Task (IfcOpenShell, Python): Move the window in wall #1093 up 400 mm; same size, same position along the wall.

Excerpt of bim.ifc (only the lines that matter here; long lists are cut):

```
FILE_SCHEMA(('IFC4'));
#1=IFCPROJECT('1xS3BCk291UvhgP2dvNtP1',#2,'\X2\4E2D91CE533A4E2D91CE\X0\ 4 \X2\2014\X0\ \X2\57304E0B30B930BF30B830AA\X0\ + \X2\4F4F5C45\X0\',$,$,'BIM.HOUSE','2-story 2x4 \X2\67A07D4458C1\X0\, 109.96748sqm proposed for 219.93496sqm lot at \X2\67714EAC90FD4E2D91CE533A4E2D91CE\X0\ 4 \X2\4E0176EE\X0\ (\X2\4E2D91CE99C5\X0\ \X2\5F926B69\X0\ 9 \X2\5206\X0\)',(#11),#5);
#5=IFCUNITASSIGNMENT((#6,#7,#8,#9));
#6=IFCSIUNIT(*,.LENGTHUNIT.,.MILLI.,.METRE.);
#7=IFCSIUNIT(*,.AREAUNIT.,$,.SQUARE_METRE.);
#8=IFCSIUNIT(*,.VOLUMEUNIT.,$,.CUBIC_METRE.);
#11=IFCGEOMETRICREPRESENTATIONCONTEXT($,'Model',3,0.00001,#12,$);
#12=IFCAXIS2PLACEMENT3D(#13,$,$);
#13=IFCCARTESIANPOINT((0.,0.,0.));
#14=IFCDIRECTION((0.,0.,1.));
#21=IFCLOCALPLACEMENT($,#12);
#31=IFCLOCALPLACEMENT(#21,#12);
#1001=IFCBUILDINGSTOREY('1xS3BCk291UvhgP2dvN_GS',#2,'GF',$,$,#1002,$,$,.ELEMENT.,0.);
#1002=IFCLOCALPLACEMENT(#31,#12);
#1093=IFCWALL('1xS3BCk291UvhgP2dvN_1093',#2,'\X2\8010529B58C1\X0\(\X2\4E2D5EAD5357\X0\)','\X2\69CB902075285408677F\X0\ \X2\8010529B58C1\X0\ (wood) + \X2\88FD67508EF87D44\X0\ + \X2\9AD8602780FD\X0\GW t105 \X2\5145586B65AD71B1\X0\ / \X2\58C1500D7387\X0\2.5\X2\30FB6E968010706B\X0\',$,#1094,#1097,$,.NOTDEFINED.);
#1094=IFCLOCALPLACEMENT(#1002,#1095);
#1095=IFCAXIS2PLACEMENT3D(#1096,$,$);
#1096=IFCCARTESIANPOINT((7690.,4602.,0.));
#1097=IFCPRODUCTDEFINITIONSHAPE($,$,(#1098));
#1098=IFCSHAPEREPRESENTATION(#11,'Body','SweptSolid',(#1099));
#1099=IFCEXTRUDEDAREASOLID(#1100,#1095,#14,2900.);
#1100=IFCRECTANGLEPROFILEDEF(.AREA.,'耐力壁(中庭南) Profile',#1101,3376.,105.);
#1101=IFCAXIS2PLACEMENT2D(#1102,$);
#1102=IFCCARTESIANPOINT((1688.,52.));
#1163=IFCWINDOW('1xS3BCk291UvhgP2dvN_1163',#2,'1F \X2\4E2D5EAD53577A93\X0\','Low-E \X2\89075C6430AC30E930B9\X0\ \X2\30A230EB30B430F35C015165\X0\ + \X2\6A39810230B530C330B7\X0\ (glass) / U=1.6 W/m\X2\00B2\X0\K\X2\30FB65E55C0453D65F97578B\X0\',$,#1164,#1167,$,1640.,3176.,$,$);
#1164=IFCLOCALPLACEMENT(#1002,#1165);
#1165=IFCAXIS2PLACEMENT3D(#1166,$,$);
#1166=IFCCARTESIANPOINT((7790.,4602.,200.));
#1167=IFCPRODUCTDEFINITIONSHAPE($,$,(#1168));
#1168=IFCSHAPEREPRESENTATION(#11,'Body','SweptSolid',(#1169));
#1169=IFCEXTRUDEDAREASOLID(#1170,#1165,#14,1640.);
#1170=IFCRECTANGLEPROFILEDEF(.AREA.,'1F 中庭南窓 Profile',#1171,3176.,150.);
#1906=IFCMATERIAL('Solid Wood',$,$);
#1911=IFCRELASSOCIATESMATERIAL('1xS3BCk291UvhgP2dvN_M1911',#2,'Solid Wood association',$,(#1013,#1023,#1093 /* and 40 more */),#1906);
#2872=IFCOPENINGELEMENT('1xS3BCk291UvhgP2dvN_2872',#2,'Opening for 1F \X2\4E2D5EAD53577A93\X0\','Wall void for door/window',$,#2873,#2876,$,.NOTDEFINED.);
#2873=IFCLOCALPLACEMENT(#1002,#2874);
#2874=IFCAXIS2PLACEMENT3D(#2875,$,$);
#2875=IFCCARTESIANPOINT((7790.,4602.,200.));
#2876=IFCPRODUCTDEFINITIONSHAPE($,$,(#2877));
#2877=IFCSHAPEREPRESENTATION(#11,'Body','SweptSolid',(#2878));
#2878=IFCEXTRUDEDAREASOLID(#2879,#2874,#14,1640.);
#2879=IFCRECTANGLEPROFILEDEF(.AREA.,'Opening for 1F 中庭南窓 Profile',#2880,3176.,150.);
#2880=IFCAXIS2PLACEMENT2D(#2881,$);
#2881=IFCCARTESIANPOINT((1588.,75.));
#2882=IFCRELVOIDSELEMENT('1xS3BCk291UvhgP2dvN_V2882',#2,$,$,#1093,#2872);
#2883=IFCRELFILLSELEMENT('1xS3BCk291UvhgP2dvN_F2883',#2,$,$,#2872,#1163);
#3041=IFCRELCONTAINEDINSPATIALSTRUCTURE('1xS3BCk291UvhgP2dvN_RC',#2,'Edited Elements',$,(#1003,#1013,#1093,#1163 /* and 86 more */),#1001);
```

```python
import numpy as np
import ifcopenshell
import ifcopenshell.api.geometry
import ifcopenshell.util.placement
import ifcopenshell.util.unit

model = ifcopenshell.open("bim.ifc")
unit_scale = ifcopenshell.util.unit.calculate_unit_scale(model)

window = model.by_id(1163)
opening = window.FillsVoids[0].RelatingOpeningElement
dz = 0.4 / unit_scale

shift = np.array([0.0, 0.0, dz])
# The window is not placed relative to its opening, so move both.
for product in (opening, window):
    matrix = ifcopenshell.util.placement.get_local_placement(product.ObjectPlacement)
    matrix[:3, 3] += shift
    ifcopenshell.api.geometry.edit_object_placement(model, product=product, matrix=matrix, is_si=False)

print(f"moved by {dz * unit_scale:+.3f} m")

model.write("bim_updated.ifc")
```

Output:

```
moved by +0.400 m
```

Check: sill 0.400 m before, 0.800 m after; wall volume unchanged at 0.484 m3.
